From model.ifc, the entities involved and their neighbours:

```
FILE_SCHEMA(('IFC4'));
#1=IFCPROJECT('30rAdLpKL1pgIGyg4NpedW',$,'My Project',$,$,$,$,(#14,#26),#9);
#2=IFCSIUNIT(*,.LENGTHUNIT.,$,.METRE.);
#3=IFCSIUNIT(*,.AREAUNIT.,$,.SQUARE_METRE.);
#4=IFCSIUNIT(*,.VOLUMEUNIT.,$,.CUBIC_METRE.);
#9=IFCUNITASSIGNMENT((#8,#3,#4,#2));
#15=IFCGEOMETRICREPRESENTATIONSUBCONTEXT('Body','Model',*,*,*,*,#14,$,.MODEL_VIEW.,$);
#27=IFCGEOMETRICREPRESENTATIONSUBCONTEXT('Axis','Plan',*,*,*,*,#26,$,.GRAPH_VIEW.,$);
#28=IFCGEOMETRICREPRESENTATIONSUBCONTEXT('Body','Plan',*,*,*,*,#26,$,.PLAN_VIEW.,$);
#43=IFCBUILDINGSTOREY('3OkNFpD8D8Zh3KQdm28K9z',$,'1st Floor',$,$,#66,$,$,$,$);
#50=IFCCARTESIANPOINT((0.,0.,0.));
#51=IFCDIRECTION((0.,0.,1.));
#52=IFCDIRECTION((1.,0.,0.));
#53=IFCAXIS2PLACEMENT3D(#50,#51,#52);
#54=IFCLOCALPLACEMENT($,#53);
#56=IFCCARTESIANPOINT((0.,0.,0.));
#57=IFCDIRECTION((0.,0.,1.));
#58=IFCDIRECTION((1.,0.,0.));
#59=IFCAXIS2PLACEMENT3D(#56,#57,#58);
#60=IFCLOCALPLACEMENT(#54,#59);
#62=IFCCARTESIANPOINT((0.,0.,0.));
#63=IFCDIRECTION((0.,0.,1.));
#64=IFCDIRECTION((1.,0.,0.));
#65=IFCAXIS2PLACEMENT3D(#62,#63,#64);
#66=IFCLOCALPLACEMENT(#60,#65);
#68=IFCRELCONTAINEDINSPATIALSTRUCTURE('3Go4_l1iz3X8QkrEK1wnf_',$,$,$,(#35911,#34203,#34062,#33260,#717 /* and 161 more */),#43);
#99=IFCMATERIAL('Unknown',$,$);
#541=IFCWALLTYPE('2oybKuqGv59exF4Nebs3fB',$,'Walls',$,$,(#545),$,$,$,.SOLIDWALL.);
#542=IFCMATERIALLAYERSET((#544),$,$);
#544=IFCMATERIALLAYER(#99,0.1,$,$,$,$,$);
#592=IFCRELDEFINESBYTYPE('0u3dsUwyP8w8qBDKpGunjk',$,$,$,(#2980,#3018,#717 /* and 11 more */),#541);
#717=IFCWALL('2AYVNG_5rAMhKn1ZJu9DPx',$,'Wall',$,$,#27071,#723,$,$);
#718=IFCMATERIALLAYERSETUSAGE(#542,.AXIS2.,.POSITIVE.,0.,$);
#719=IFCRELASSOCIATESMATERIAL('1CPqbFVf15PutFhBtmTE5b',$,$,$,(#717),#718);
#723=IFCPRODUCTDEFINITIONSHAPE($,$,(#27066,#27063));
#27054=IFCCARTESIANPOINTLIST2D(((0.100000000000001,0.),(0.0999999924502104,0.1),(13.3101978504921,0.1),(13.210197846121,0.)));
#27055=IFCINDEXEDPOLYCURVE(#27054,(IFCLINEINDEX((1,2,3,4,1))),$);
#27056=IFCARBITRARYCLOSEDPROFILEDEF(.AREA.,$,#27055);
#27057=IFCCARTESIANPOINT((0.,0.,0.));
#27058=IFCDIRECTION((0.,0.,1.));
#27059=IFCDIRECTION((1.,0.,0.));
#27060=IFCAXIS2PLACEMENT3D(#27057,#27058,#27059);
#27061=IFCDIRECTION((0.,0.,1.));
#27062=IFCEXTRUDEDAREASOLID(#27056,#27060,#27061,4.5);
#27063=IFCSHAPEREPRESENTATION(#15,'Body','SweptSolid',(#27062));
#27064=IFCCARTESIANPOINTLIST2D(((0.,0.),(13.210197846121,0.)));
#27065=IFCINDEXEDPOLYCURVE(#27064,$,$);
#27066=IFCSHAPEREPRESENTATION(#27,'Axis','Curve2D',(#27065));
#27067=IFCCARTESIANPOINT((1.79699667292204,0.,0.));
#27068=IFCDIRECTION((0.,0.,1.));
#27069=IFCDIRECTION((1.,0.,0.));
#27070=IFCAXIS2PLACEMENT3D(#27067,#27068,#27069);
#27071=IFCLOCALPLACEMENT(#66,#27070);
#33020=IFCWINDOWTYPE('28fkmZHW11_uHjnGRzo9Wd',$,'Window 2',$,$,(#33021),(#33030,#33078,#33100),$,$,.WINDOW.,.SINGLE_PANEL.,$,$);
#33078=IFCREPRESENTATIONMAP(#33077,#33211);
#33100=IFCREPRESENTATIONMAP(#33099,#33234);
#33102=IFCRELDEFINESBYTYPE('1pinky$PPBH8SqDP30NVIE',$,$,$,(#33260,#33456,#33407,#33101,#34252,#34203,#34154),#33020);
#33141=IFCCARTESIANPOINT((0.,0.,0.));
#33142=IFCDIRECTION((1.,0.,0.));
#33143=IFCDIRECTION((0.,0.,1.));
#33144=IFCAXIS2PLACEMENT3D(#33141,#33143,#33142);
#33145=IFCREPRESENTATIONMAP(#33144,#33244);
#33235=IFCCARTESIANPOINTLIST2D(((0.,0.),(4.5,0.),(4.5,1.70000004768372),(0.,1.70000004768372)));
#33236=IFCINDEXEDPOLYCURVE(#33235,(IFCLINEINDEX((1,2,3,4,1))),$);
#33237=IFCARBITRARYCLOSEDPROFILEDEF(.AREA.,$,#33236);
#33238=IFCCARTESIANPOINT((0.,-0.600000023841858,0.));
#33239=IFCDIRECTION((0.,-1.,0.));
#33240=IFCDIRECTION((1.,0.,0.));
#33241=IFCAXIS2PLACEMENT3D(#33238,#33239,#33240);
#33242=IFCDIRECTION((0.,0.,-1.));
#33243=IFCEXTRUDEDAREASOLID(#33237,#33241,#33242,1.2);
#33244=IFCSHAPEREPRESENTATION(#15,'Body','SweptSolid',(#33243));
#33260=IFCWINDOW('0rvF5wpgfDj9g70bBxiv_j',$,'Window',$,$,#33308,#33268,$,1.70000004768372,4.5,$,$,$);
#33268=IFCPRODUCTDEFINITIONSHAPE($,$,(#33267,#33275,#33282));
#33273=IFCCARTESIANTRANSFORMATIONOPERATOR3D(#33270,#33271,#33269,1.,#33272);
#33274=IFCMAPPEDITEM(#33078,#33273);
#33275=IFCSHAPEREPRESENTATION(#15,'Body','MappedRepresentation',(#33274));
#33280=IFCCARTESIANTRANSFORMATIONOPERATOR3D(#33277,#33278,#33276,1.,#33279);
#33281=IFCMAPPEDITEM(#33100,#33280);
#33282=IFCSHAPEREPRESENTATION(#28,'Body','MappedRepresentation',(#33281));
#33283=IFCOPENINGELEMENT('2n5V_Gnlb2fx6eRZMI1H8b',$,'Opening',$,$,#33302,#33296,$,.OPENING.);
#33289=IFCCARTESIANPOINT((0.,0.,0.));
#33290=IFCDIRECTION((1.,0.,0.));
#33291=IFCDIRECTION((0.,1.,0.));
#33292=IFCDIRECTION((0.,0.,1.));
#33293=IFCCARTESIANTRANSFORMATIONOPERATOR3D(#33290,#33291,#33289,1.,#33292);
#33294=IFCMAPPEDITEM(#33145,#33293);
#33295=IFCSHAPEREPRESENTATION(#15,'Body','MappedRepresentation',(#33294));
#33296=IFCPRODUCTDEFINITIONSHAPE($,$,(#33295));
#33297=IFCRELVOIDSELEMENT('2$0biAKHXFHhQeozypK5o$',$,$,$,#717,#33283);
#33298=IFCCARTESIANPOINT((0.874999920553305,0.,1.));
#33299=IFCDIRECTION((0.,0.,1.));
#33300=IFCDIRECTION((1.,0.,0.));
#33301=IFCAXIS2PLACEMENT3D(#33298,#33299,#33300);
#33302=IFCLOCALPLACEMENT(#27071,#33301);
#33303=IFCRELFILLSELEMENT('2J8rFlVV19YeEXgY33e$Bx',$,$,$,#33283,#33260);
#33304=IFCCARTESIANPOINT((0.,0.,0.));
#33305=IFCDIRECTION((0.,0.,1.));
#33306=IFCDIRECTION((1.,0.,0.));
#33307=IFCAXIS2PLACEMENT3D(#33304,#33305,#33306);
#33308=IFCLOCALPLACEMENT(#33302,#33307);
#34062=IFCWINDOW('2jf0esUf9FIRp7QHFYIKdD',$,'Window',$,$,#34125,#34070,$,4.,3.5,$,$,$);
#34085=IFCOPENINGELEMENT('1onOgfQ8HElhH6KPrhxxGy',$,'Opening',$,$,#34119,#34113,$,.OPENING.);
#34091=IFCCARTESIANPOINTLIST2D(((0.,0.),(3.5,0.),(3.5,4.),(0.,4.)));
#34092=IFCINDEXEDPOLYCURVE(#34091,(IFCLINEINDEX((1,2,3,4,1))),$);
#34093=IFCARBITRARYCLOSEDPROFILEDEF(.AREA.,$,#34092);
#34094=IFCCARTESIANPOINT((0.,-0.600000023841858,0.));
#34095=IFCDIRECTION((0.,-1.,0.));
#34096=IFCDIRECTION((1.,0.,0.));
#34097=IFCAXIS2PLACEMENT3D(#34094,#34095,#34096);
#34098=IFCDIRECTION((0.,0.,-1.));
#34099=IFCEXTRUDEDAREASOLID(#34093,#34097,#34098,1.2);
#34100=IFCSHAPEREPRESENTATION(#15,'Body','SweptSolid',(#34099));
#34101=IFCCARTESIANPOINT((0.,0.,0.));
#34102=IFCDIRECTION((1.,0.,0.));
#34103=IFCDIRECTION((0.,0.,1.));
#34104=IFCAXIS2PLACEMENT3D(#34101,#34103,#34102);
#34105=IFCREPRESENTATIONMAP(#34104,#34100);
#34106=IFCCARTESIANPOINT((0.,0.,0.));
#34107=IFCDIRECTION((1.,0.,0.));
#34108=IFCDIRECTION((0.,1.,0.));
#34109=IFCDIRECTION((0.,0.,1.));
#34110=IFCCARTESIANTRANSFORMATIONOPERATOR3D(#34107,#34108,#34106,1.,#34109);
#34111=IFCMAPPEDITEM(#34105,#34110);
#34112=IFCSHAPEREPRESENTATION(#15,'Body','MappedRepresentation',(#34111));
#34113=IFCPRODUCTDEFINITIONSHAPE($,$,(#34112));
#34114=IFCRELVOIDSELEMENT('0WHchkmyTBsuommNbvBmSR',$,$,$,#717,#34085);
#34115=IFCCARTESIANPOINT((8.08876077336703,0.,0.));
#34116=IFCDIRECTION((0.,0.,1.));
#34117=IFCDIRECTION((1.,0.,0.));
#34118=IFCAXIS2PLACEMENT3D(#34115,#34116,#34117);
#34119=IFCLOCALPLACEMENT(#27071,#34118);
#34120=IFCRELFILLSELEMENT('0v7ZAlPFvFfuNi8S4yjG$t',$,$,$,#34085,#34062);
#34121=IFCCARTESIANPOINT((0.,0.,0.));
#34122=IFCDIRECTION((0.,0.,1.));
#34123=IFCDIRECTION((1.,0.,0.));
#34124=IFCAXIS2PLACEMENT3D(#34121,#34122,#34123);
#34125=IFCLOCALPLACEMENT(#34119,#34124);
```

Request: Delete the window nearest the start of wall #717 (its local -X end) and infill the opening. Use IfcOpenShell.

```python
import ifcopenshell
import ifcopenshell.api.feature
import ifcopenshell.api.root
import ifcopenshell.geom
import ifcopenshell.util.shape

model = ifcopenshell.open("model.ifc")
settings = ifcopenshell.geom.settings()


def volume(element):
    """Net volume in cubic metres, openings subtracted."""
    shape = ifcopenshell.geom.create_shape(settings, element)
    return ifcopenshell.util.shape.get_volume(shape.geometry)


window = model.by_guid("0rvF5wpgfDj9g70bBxiv_j")
opening = window.FillsVoids[0].RelatingOpeningElement
wall = opening.VoidsElements[0].RelatingBuildingElement
before = volume(wall)

ifcopenshell.api.root.remove_product(model, product=window)
ifcopenshell.api.feature.remove_feature(model, feature=opening)

after = volume(wall)

print(f"wall volume {before:.3f} -> {after:.3f} m3")

model.write("model-out.ifc")
```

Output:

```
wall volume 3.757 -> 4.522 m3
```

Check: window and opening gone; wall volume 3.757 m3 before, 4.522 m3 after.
